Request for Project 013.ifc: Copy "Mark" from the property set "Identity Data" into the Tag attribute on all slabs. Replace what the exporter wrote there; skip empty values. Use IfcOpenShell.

First a look at what the model holds.

```python
import ifcopenshell
import ifcopenshell.util.element

model = ifcopenshell.open("Project 013.ifc")
print(model.schema)
slabs = model.by_type("IfcSlab")
print(len(slabs), "slabs")
for e in slabs[:8]:
    source = ifcopenshell.util.element.get_pset(e, "Identity Data", "Mark")
    target = e.Tag
    print(e.id(), repr(source), repr(target), sep=" | ")
```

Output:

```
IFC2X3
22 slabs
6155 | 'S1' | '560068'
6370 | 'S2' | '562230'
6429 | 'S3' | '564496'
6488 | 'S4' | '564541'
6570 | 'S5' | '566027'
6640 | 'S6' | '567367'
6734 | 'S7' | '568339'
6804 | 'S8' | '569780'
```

```python
import ifcopenshell
import ifcopenshell.util.element

model = ifcopenshell.open("Project 013.ifc")

count = 0
for e in model.by_type("IfcSlab"):
    value = ifcopenshell.util.element.get_pset(e, "Identity Data", "Mark")
    current = e.Tag
    if not value or not value.strip() or current == value:
        continue
    e.Tag = value
    count += 1

print(count, "slabs updated")

model.write("Project 013_updated.ifc")
```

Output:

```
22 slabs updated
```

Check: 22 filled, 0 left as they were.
